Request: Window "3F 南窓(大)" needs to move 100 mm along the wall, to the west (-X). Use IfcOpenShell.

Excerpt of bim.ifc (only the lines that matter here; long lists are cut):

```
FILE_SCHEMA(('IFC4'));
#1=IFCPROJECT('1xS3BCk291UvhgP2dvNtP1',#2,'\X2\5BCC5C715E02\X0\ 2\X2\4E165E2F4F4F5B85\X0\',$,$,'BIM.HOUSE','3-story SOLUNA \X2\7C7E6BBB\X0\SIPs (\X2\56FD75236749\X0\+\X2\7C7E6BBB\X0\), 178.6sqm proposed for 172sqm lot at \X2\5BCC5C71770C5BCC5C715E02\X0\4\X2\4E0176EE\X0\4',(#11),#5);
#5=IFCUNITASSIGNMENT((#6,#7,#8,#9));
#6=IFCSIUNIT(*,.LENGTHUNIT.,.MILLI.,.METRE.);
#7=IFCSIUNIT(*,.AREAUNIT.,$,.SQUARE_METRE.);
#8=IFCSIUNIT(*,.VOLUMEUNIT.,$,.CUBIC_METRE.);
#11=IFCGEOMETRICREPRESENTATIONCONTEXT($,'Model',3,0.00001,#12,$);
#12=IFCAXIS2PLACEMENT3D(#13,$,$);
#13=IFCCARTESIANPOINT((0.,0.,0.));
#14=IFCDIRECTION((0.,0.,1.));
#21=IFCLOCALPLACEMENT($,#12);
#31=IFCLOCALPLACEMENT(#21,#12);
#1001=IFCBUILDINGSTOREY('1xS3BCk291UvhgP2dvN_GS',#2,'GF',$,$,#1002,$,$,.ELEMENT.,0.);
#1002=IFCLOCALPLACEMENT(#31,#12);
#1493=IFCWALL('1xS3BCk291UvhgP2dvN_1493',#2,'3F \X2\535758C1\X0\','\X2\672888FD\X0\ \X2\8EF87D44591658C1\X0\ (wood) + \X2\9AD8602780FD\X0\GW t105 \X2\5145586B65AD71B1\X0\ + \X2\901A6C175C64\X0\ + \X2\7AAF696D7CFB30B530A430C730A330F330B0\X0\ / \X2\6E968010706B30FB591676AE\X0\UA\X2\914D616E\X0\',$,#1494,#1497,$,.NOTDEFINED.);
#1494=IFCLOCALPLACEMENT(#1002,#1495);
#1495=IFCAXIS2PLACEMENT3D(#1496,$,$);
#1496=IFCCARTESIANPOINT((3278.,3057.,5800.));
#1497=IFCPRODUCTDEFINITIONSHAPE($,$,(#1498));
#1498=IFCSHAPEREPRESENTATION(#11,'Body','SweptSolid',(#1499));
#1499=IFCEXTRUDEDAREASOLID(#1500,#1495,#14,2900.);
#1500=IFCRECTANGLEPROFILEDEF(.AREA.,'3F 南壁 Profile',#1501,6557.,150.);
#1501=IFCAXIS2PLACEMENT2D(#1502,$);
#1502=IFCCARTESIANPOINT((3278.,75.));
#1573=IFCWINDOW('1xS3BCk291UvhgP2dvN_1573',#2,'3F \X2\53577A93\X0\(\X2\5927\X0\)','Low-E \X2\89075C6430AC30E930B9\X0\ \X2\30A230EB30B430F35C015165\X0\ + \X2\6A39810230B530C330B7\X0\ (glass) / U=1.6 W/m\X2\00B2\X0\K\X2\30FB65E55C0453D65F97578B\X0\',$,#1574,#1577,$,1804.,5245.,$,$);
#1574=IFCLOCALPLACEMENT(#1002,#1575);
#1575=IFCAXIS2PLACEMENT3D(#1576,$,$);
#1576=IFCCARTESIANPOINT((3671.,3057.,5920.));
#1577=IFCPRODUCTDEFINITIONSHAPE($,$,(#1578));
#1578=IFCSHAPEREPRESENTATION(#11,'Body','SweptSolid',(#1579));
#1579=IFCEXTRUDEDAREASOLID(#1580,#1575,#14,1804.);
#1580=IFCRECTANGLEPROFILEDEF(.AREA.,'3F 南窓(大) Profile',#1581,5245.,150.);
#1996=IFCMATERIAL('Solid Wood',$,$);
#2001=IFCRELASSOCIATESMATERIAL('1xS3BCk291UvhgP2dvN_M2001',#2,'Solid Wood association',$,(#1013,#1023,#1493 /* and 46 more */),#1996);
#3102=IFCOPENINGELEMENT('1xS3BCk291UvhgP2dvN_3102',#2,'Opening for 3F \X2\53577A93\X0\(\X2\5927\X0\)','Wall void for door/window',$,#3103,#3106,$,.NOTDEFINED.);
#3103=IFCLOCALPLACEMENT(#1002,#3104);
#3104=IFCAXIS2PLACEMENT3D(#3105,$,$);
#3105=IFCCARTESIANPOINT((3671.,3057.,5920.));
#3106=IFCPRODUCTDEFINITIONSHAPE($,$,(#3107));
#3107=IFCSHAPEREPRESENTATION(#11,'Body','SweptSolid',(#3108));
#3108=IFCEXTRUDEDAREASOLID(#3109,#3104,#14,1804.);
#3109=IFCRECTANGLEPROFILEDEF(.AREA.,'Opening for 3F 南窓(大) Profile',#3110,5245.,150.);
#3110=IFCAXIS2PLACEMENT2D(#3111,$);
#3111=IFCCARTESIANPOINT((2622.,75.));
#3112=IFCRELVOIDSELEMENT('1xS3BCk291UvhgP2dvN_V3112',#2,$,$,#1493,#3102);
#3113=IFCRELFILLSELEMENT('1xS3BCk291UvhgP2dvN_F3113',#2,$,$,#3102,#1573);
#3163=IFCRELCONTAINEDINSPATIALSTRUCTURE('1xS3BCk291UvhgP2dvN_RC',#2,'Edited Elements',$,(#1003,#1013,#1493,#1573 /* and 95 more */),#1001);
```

```python
import ifcopenshell
import ifcopenshell.api.geometry
import ifcopenshell.util.placement

model = ifcopenshell.open("bim.ifc")

window = model.by_guid("1xS3BCk291UvhgP2dvN_1573")
opening = window.FillsVoids[0].RelatingOpeningElement
wall = opening.VoidsElements[0].RelatingBuildingElement

wall_matrix = ifcopenshell.util.placement.get_local_placement(wall.ObjectPlacement)
shift = wall_matrix[:3, 0] * -100.0
before = ifcopenshell.util.placement.get_local_placement(window.ObjectPlacement)[:3, 3].copy()

# The window is not placed relative to its opening, so move both.
for product in (opening, window):
    matrix = ifcopenshell.util.placement.get_local_placement(product.ObjectPlacement)
    matrix[:3, 3] += shift
    ifcopenshell.api.geometry.edit_object_placement(model, product=product, matrix=matrix, is_si=False)

after = ifcopenshell.util.placement.get_local_placement(window.ObjectPlacement)[:3, 3]
print("window moved by", (after - before).round(3) + 0.0)

model.write("bim_updated.ifc")
```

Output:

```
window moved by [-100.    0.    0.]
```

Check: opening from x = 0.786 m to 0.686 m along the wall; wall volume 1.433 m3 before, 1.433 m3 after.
